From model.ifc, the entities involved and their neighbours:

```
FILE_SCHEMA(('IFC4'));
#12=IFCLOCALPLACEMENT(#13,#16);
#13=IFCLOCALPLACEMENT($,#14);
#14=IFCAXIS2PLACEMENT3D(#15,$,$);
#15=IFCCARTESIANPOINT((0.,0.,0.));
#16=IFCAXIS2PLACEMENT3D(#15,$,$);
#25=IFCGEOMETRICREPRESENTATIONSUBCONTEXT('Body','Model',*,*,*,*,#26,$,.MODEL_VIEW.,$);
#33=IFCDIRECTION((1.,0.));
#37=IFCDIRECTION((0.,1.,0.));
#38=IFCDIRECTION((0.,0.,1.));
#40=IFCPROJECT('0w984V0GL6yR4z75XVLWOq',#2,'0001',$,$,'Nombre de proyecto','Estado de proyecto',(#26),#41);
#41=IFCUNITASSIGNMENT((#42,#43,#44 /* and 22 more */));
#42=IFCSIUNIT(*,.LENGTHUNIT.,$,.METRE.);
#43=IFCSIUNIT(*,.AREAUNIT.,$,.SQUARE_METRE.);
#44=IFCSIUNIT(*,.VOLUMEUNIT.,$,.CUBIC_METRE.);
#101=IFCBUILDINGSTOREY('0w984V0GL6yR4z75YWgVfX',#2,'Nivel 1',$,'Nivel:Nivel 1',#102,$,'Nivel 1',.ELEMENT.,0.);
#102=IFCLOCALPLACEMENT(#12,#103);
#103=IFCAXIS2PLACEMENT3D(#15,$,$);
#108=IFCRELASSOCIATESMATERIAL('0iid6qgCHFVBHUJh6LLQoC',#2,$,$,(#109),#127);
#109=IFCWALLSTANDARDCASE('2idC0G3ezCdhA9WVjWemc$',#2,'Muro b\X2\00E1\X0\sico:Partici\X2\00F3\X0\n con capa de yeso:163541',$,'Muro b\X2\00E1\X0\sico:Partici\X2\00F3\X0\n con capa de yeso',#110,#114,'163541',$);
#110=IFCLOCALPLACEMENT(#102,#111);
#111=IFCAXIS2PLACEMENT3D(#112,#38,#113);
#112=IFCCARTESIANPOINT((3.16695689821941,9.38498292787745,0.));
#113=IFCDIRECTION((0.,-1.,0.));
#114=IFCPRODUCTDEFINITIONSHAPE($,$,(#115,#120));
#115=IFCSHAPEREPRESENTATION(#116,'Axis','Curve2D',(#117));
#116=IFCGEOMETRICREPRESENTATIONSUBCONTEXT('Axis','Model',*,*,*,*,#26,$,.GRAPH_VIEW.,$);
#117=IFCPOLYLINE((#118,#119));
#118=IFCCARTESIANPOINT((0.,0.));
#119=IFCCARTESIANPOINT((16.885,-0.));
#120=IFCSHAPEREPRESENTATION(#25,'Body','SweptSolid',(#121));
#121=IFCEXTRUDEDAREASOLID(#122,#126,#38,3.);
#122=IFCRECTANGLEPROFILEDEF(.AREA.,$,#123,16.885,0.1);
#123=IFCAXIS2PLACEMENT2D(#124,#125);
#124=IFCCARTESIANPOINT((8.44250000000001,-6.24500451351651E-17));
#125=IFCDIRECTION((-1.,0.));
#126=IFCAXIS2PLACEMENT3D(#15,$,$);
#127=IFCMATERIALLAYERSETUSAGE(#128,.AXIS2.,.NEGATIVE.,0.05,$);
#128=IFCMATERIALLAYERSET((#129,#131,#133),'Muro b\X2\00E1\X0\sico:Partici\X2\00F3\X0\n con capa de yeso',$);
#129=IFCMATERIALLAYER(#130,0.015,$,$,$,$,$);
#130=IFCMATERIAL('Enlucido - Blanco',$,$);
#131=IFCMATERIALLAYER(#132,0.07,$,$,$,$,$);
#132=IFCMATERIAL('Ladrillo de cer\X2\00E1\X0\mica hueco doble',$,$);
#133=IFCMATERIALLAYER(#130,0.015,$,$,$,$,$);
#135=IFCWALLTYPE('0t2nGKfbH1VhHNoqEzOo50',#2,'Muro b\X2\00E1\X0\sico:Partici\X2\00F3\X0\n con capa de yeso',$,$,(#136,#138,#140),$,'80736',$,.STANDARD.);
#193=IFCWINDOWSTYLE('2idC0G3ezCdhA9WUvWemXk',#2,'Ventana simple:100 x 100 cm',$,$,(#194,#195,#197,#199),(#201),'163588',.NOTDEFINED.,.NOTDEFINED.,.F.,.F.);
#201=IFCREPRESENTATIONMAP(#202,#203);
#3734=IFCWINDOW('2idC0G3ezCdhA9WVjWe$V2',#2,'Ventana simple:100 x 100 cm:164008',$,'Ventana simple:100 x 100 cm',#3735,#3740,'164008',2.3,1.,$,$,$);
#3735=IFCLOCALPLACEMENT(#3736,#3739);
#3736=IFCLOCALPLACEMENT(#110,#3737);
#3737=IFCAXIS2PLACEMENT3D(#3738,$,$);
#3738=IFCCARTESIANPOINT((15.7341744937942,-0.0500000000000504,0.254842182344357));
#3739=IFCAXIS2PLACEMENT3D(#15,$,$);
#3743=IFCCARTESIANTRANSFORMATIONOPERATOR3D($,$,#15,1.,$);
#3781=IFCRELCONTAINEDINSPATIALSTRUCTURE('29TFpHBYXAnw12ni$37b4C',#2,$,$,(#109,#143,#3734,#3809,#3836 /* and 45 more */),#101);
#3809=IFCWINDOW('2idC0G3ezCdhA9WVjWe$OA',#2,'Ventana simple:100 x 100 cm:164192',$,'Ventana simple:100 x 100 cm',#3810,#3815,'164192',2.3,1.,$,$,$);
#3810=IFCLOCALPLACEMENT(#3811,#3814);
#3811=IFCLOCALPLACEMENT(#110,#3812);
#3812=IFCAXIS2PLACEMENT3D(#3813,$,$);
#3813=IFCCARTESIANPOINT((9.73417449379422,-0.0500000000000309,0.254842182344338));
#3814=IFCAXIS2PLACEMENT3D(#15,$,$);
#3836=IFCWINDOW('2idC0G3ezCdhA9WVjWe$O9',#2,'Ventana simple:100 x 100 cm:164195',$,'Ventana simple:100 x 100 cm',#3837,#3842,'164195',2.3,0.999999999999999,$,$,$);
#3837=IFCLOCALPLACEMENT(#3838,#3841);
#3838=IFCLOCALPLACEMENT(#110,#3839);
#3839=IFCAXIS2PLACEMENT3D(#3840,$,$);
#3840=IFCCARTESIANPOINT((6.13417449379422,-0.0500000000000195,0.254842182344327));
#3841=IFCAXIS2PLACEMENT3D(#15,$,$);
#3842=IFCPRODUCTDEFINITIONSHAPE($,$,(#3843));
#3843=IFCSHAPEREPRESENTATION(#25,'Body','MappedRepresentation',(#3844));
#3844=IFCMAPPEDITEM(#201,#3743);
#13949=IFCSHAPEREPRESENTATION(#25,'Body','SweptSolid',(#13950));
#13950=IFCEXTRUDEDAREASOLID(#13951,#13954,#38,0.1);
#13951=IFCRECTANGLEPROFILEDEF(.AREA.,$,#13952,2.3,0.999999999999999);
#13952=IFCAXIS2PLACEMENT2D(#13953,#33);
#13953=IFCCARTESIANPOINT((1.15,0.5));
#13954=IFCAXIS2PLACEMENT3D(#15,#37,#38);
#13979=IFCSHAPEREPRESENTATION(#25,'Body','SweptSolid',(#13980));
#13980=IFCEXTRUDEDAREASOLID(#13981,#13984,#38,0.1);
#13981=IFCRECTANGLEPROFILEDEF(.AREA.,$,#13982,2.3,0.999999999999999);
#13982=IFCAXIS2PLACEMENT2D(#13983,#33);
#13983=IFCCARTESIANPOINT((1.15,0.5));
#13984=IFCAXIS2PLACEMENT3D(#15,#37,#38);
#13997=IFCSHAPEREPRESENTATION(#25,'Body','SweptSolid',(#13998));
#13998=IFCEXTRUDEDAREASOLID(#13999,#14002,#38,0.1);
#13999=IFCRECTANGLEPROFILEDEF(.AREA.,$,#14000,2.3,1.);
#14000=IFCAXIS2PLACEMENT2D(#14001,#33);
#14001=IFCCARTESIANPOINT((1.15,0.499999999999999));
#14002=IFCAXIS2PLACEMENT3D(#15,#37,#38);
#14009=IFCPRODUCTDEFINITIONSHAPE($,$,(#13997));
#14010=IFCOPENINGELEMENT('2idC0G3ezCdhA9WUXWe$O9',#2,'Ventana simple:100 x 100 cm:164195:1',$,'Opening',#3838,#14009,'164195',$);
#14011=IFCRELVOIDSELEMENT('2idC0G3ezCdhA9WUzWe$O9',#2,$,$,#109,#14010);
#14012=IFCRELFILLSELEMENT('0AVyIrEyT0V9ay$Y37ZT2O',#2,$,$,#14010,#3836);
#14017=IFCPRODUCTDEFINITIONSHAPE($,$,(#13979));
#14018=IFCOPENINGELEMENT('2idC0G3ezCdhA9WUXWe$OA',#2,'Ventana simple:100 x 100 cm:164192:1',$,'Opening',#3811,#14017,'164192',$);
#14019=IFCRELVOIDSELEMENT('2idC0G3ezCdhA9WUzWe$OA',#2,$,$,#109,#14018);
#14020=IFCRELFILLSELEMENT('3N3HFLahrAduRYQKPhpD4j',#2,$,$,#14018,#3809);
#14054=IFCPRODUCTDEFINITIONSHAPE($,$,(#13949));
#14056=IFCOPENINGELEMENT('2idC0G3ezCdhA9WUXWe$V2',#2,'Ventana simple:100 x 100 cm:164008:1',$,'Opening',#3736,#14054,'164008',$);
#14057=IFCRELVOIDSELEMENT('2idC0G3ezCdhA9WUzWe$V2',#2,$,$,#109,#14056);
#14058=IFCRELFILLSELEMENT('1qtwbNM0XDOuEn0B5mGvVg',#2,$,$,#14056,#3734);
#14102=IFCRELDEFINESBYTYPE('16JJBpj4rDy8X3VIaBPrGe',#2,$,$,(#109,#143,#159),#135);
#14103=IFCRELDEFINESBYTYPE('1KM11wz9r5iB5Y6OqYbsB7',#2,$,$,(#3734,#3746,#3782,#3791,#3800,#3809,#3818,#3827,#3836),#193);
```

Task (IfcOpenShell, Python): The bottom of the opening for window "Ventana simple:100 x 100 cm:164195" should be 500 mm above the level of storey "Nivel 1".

```python
import numpy as np
import ifcopenshell
import ifcopenshell.api.geometry
import ifcopenshell.geom
import ifcopenshell.util.element
import ifcopenshell.util.placement
import ifcopenshell.util.shape
import ifcopenshell.util.unit

model = ifcopenshell.open("model.ifc")
unit_scale = ifcopenshell.util.unit.calculate_unit_scale(model)

window = model.by_guid("2idC0G3ezCdhA9WVjWe$O9")
opening = window.FillsVoids[0].RelatingOpeningElement
storey = ifcopenshell.util.element.get_container(window, ifc_class="IfcBuildingStorey")
level = ifcopenshell.util.placement.get_local_placement(storey.ObjectPlacement)[2, 3]

# The opening's origin need not be at the sill, so measure its lowest point.
shape = ifcopenshell.geom.create_shape(ifcopenshell.geom.settings(), opening)
bottom = ifcopenshell.util.shape.get_shape_bottom_elevation(shape, shape.geometry) / unit_scale
dz = level + 0.5 - bottom

shift = np.array([0.0, 0.0, dz])
# The window is placed relative to its opening, so it follows when the opening moves.
matrix = ifcopenshell.util.placement.get_local_placement(opening.ObjectPlacement)
matrix[:3, 3] += shift
ifcopenshell.api.geometry.edit_object_placement(
    model, product=opening, matrix=matrix, is_si=False, should_transform_children=True
)

print(f"moved by {dz * unit_scale:+.3f} m")

model.write("model_v2.ifc")
```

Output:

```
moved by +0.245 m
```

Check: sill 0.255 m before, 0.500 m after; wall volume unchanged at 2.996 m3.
